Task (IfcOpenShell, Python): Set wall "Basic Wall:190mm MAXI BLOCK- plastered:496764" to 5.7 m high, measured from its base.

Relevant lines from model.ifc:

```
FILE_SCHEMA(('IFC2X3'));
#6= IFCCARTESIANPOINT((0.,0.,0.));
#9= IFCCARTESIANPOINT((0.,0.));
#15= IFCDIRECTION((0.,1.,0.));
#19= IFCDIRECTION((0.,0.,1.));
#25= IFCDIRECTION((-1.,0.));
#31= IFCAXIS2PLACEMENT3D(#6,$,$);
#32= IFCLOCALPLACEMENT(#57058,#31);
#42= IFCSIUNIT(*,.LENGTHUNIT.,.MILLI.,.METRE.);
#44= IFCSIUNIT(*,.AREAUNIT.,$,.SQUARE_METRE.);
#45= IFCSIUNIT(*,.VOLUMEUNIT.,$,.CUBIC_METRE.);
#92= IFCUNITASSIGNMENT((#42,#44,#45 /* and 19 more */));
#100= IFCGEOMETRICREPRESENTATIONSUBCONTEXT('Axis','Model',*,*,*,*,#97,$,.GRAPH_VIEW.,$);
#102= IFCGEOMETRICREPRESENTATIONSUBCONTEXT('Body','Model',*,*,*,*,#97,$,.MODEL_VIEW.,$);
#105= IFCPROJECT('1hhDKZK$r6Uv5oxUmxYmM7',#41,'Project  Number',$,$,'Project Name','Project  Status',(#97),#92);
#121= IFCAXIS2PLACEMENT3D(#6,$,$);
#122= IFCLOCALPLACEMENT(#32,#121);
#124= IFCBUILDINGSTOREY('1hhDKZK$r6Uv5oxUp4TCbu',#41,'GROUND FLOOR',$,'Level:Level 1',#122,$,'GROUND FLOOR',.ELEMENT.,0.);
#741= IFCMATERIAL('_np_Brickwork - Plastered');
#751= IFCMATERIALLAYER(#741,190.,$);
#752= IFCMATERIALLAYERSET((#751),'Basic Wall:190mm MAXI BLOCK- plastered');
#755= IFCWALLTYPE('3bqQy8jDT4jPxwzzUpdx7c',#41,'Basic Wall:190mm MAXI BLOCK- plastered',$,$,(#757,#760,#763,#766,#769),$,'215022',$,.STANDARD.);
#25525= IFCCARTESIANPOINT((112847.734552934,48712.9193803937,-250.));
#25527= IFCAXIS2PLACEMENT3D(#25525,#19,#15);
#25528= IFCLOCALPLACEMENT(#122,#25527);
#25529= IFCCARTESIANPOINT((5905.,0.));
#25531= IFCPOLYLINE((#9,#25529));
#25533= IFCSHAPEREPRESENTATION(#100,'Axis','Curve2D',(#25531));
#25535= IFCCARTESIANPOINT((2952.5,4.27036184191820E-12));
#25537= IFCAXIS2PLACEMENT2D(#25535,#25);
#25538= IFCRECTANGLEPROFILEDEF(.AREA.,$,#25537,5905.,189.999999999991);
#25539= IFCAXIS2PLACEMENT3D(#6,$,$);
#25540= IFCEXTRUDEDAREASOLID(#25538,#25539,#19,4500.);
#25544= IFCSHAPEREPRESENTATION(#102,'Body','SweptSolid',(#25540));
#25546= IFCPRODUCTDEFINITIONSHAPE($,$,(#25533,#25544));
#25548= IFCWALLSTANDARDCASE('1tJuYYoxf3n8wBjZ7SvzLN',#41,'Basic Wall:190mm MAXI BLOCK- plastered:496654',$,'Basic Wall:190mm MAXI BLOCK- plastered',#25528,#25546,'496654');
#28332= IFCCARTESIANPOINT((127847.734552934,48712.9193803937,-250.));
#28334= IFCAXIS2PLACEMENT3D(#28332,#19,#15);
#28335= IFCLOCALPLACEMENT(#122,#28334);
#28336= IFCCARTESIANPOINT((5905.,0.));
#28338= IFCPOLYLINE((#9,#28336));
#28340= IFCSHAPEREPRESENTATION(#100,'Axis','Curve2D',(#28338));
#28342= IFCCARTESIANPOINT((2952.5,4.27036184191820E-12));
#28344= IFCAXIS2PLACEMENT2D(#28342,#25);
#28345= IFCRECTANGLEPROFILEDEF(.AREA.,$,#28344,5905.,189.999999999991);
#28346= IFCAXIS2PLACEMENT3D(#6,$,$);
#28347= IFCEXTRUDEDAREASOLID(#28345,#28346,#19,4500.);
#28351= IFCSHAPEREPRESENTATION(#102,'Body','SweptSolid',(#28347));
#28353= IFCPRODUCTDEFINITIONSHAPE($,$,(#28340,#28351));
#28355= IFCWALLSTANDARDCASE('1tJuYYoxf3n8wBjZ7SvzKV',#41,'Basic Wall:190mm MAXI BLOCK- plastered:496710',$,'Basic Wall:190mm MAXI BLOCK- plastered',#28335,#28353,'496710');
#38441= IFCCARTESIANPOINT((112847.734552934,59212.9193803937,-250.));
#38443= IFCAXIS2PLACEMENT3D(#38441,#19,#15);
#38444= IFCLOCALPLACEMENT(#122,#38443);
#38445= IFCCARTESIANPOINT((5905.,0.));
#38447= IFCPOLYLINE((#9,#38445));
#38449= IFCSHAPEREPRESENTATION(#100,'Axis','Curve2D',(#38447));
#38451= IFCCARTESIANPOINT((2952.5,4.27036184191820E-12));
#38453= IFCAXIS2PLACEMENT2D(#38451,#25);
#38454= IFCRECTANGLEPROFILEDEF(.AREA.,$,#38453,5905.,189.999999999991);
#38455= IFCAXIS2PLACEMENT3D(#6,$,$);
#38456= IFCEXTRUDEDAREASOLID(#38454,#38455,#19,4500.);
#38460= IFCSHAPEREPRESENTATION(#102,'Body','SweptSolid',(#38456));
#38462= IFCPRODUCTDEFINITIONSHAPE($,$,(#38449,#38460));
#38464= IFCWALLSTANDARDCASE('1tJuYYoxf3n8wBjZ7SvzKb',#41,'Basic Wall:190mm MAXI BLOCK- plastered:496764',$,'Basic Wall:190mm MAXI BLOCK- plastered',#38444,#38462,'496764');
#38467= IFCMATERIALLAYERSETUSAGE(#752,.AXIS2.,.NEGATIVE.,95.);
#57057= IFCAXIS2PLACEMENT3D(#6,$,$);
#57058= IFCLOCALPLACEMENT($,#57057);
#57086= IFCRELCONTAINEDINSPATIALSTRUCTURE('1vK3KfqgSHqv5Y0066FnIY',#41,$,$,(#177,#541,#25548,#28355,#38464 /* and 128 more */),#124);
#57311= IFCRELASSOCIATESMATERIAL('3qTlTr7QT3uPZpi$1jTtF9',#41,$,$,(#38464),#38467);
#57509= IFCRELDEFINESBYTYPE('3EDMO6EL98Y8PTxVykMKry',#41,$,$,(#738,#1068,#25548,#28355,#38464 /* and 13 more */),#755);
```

```python
import ifcopenshell
import ifcopenshell.geom
import ifcopenshell.util.representation
import ifcopenshell.util.shape
import ifcopenshell.util.unit

model = ifcopenshell.open("model.ifc")
unit_scale = ifcopenshell.util.unit.calculate_unit_scale(model)
settings = ifcopenshell.geom.settings()


def volume(element):
    """Net volume in cubic metres, openings subtracted."""
    shape = ifcopenshell.geom.create_shape(settings, element)
    return ifcopenshell.util.shape.get_volume(shape.geometry)


wall = model.by_guid("1tJuYYoxf3n8wBjZ7SvzKb")
before = volume(wall)

body = ifcopenshell.util.representation.get_representation(wall, "Model", "Body")
solid = body.Items[0]
old_height = solid.Depth
solid.Depth = 5.7 / unit_scale
after = volume(wall)

print(f"height {old_height:g} -> {solid.Depth:g}, volume {before:.3f} -> {after:.3f} m3")

model.write("model_v2.ifc")
```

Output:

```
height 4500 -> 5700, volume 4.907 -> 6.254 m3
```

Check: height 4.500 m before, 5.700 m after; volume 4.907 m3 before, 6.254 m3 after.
